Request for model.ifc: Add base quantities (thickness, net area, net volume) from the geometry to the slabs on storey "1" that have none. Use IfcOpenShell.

First a look at what the model holds.

```python
import ifcopenshell
import ifcopenshell.util.element
import ifcopenshell.util.unit

model = ifcopenshell.open("model.ifc")
print(model.schema)
for unit_type in ("LENGTHUNIT", "AREAUNIT", "VOLUMEUNIT"):
    print(unit_type, ifcopenshell.util.unit.calculate_unit_scale(model, unit_type))
storey = next(s for s in model.by_type("IfcBuildingStorey") if s.Name == "1")
slabs = [e for e in ifcopenshell.util.element.get_decomposition(storey) if e.is_a("IfcSlab")]
for e in sorted(slabs, key=lambda e: e.id()):
    print(e.id(), e.is_a(), e.Name, list(ifcopenshell.util.element.get_psets(e, qtos_only=True)), sep=" | ")
```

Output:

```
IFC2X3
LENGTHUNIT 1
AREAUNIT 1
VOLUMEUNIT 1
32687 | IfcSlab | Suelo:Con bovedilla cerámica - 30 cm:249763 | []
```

```python
import ifcopenshell
import ifcopenshell.api.pset
import ifcopenshell.geom
import ifcopenshell.util.element
import ifcopenshell.util.shape
import ifcopenshell.util.unit

model = ifcopenshell.open("model.ifc")
unit_scale = ifcopenshell.util.unit.calculate_unit_scale(model)
area_scale = ifcopenshell.util.unit.calculate_unit_scale(model, "AREAUNIT")
volume_scale = ifcopenshell.util.unit.calculate_unit_scale(model, "VOLUMEUNIT")
settings = ifcopenshell.geom.settings()

storey = next(s for s in model.by_type("IfcBuildingStorey") if s.Name == "1")
slabs = [e for e in ifcopenshell.util.element.get_decomposition(storey) if e.is_a("IfcSlab")]

for e in sorted(slabs, key=lambda e: e.id()):
    if ifcopenshell.util.element.get_psets(e, qtos_only=True, should_inherit=False):
        continue
    # Geometry comes back in metres, in the element's own axes.
    shape = ifcopenshell.geom.create_shape(settings, e)
    values = {
        "Width": ifcopenshell.util.shape.get_z(shape.geometry) / unit_scale,
        "NetArea": ifcopenshell.util.shape.get_footprint_area(shape.geometry) / area_scale,
        "NetVolume": ifcopenshell.util.shape.get_volume(shape.geometry) / volume_scale,
    }
    qto = ifcopenshell.api.pset.add_qto(model, product=e, name="BaseQuantities")
    ifcopenshell.api.pset.edit_qto(model, qto=qto, properties=values)
    print(e.id(), {k: round(v, 3) for k, v in values.items()})

model.write("model-out.ifc")
```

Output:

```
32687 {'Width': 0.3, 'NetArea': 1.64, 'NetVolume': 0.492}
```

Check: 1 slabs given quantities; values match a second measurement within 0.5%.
